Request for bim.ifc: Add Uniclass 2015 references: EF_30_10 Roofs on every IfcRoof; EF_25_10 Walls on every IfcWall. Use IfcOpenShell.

First a look at what the model holds.

```python
import ifcopenshell

model = ifcopenshell.open("bim.ifc")
print(model.schema)
print("classifications:", [c.Name for c in model.by_type("IfcClassification")])
for ifc_class in ("IfcDoor", "IfcRoof", "IfcStair", "IfcWall", "IfcWindow"):
    print(ifc_class, len(model.by_type(ifc_class)))
```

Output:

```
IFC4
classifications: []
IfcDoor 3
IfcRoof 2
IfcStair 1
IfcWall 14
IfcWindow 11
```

```python
import ifcopenshell
import ifcopenshell.api.classification

model = ifcopenshell.open("bim.ifc")

system = ifcopenshell.api.classification.add_classification(model, classification="Uniclass 2015")

codes = {
    "IfcRoof": ("EF_30_10", "Roofs"),
    "IfcWall": ("EF_25_10", "Walls"),
}
for ifc_class, (code, name) in codes.items():
    products = model.by_type(ifc_class)
    ifcopenshell.api.classification.add_reference(
        model, products=products, classification=system, identification=code, name=name
    )
    print(code, len(products))

model.write("bim_rev.ifc")
```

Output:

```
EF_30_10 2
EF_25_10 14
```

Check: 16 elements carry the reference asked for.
